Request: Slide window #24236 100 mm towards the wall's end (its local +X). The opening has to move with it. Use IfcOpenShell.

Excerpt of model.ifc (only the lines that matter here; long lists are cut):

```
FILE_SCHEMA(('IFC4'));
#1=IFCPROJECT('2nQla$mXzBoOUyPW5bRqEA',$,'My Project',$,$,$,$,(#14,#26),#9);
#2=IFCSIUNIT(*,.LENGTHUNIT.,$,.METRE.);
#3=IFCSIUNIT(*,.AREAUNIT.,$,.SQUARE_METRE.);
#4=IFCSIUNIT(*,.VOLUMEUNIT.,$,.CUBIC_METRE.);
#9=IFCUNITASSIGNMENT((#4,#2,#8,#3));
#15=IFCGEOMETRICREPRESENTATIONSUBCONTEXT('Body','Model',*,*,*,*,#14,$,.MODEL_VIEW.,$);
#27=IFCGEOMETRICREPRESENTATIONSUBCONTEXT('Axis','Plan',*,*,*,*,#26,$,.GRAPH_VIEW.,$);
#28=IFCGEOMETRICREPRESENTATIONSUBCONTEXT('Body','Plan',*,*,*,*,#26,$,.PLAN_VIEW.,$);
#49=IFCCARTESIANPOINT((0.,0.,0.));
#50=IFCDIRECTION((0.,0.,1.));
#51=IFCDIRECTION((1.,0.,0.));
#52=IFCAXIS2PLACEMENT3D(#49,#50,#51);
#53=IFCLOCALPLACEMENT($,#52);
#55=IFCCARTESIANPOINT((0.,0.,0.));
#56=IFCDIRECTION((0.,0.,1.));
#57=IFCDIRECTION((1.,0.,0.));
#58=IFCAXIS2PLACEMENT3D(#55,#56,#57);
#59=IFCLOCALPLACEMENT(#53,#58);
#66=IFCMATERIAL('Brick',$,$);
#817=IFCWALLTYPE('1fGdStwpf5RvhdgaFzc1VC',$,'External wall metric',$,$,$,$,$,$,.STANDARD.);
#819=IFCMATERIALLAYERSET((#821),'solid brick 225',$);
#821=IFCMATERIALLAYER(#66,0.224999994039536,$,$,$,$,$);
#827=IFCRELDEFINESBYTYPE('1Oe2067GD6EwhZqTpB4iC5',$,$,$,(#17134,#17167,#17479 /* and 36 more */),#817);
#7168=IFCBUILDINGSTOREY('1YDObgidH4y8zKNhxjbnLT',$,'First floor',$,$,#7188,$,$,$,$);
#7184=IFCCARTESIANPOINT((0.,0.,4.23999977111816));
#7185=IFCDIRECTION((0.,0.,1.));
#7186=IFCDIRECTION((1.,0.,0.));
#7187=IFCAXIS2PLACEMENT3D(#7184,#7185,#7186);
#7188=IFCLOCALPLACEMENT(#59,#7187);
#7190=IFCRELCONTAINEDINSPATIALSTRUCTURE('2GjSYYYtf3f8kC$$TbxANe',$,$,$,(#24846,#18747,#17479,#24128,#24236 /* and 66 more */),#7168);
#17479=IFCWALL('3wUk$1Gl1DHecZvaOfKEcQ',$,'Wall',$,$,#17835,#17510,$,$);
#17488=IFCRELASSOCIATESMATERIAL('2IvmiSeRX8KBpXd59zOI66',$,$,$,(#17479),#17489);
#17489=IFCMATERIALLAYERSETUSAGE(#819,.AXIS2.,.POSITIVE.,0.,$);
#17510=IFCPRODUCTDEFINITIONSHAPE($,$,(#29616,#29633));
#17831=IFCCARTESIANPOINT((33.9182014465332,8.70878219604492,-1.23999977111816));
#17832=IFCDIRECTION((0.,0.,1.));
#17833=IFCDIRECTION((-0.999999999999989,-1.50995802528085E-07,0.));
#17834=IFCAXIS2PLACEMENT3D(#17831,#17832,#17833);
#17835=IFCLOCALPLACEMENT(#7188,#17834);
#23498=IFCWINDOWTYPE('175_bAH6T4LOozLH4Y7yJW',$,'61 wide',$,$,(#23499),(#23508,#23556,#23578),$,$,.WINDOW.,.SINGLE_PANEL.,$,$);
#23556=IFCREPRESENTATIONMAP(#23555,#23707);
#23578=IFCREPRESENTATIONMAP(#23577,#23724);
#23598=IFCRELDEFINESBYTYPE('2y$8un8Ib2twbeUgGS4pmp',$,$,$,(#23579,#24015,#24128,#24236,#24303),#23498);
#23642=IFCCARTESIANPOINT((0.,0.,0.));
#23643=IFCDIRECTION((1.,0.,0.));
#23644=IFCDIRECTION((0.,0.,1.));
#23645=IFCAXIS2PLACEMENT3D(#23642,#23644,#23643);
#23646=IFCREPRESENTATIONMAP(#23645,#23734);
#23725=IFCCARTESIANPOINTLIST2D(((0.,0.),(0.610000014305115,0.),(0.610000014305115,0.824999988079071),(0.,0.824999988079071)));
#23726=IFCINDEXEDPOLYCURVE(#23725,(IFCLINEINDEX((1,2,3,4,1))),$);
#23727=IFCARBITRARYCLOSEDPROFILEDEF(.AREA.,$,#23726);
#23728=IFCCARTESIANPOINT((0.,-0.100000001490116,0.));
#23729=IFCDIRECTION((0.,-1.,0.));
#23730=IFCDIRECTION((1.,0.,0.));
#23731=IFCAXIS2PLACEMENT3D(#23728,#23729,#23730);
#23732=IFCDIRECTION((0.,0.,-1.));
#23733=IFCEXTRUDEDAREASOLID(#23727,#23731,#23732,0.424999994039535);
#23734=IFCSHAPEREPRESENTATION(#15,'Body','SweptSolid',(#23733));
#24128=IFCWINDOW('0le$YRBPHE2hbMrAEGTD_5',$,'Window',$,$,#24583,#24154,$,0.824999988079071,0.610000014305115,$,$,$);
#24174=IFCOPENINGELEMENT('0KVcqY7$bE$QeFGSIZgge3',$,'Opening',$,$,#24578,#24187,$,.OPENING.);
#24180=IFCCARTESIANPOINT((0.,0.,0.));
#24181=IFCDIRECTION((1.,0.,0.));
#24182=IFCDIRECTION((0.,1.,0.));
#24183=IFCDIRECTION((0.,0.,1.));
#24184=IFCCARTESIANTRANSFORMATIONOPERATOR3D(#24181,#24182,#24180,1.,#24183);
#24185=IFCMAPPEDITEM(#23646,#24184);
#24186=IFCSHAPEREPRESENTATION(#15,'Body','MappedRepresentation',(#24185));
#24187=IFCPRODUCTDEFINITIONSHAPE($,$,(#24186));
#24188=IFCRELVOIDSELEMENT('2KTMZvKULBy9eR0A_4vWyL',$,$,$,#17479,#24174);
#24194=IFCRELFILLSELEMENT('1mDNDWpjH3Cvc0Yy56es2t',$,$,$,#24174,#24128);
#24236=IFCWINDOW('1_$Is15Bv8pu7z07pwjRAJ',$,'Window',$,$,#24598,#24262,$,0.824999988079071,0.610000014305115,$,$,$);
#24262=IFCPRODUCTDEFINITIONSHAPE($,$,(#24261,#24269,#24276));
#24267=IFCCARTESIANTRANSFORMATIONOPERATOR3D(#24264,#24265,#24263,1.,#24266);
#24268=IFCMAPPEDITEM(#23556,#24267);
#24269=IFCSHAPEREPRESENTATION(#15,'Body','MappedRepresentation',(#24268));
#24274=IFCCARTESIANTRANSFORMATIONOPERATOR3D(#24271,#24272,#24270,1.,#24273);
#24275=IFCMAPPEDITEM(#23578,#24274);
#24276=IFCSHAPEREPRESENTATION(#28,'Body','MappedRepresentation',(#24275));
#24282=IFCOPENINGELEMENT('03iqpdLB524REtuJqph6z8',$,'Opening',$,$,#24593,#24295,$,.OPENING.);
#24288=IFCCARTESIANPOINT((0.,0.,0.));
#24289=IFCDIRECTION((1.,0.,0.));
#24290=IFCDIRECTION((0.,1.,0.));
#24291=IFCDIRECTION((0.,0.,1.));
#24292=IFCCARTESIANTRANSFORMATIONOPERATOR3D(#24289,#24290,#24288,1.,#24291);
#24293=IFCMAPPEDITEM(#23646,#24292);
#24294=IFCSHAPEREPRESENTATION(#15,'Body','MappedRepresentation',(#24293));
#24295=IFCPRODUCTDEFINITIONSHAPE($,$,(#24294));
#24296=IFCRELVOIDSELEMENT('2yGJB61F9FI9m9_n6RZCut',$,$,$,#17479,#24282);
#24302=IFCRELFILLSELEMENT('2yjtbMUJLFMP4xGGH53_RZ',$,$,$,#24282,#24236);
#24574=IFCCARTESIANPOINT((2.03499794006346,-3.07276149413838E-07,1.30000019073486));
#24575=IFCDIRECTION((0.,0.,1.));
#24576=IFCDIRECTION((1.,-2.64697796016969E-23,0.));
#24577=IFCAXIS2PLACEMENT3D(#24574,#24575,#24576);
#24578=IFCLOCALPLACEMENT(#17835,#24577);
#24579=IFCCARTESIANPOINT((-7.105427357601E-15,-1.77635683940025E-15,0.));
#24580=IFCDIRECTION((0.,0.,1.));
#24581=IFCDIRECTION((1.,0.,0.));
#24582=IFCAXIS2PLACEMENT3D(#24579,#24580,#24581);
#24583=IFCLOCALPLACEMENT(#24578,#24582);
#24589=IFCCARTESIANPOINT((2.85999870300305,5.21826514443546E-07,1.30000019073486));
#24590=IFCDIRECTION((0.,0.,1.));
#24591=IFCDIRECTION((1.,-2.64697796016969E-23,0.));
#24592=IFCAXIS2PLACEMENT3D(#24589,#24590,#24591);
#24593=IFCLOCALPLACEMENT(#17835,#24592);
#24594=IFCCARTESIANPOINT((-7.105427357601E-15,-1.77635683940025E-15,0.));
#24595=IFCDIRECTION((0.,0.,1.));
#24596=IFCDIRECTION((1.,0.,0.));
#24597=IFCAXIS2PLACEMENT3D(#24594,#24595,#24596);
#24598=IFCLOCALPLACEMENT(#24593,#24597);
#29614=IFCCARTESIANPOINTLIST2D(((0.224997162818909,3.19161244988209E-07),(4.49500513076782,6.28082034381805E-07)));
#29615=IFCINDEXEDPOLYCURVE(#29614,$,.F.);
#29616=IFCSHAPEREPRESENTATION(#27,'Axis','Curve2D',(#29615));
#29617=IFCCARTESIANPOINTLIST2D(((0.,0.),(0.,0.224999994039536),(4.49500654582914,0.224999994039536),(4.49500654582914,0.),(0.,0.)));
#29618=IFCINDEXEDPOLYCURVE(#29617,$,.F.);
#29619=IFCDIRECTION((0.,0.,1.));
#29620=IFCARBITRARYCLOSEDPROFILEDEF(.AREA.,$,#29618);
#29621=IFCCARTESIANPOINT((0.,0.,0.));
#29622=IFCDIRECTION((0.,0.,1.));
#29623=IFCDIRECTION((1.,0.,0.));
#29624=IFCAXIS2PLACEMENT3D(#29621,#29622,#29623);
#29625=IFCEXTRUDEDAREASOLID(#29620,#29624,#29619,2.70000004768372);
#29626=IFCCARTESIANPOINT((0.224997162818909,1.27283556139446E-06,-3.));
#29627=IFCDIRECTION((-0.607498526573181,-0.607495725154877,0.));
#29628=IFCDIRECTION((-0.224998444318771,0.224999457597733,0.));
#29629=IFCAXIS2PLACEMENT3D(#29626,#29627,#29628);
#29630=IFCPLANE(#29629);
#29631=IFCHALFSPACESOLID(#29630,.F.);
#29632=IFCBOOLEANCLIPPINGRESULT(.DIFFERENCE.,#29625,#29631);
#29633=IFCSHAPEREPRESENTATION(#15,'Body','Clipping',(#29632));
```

```python
import ifcopenshell
import ifcopenshell.api.geometry
import ifcopenshell.util.placement
import ifcopenshell.util.unit

model = ifcopenshell.open("model.ifc")
unit_scale = ifcopenshell.util.unit.calculate_unit_scale(model)

window = model.by_guid("1_$Is15Bv8pu7z07pwjRAJ")
opening = window.FillsVoids[0].RelatingOpeningElement
wall = opening.VoidsElements[0].RelatingBuildingElement

wall_matrix = ifcopenshell.util.placement.get_local_placement(wall.ObjectPlacement)
shift = wall_matrix[:3, 0] * 0.1 / unit_scale
before = ifcopenshell.util.placement.get_local_placement(window.ObjectPlacement)[:3, 3].copy()

# The window is placed relative to its opening, so it follows when the opening moves.
matrix = ifcopenshell.util.placement.get_local_placement(opening.ObjectPlacement)
matrix[:3, 3] += shift
ifcopenshell.api.geometry.edit_object_placement(
    model, product=opening, matrix=matrix, is_si=False, should_transform_children=True
)

after = ifcopenshell.util.placement.get_local_placement(window.ObjectPlacement)[:3, 3]
print("window moved by", (after - before).round(3) + 0.0)

model.write("model-out.ifc")
```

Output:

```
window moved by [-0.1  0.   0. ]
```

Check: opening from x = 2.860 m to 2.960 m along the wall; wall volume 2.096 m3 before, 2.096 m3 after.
